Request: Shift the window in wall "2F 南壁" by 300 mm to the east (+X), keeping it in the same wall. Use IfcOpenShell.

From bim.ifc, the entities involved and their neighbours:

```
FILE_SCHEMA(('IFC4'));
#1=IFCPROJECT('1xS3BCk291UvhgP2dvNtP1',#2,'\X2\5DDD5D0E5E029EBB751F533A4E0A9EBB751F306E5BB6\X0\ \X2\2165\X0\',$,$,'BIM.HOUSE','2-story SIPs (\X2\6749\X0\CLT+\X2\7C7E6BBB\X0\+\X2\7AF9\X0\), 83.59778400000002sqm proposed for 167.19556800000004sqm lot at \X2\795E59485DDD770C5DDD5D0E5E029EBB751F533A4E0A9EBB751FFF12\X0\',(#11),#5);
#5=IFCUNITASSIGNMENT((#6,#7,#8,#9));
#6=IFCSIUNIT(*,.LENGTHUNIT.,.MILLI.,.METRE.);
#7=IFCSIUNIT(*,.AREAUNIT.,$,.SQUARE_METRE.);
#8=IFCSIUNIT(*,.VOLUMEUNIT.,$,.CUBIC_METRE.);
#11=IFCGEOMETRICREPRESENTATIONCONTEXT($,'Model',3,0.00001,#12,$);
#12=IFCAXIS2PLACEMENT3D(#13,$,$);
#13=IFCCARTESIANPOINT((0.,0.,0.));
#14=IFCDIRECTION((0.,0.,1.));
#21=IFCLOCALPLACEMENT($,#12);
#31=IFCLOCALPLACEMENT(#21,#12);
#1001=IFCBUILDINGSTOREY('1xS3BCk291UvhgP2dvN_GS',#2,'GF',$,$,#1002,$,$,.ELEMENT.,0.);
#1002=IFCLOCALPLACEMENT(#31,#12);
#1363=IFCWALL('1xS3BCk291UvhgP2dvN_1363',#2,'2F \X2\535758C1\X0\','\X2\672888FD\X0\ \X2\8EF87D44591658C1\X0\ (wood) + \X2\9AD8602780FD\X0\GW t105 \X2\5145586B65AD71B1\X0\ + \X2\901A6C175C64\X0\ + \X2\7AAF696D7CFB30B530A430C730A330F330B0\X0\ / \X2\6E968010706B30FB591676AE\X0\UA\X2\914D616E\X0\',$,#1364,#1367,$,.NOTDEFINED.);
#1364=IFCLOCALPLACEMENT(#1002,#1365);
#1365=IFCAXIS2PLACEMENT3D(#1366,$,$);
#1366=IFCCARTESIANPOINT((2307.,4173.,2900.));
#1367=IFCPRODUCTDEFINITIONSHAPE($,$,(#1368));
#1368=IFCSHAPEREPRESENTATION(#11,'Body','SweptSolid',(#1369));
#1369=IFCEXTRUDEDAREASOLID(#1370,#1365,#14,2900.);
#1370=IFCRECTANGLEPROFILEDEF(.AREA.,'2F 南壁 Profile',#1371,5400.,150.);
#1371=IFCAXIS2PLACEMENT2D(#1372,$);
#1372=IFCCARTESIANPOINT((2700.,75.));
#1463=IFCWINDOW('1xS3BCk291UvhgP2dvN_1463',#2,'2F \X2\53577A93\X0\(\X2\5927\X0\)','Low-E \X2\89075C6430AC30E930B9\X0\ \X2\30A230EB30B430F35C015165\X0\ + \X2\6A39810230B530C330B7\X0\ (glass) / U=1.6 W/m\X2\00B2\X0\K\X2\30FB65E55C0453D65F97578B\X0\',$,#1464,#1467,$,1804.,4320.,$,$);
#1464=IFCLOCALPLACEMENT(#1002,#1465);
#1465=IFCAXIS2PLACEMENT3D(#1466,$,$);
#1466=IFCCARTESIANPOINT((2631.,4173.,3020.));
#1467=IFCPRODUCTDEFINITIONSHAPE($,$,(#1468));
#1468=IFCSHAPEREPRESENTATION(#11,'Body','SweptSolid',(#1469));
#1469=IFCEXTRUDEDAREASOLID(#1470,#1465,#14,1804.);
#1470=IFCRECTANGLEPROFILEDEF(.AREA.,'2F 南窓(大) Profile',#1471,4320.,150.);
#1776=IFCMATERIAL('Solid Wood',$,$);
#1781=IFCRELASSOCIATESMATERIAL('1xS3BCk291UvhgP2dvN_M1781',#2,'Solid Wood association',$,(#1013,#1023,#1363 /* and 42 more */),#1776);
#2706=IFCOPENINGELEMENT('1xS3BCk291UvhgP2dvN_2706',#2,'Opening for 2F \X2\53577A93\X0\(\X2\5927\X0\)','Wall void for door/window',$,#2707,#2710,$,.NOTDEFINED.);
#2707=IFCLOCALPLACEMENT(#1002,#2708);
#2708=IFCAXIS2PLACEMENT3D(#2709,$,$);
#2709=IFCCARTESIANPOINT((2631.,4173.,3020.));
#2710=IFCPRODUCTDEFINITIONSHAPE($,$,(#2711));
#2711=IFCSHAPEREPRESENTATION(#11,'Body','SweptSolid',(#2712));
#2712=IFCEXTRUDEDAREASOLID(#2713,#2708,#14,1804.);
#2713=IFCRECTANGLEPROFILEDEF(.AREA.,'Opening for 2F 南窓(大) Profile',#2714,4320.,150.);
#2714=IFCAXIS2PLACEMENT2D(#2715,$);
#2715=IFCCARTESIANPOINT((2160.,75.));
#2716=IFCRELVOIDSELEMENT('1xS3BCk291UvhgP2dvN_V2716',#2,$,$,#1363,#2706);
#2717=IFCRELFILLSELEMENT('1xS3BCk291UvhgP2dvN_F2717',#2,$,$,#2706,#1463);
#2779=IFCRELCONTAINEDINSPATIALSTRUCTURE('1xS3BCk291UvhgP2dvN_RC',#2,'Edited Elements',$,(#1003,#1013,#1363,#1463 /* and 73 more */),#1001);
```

```python
import ifcopenshell
import ifcopenshell.api.geometry
import ifcopenshell.util.placement

model = ifcopenshell.open("bim.ifc")

window = model.by_id(1463)
opening = window.FillsVoids[0].RelatingOpeningElement
wall = opening.VoidsElements[0].RelatingBuildingElement

wall_matrix = ifcopenshell.util.placement.get_local_placement(wall.ObjectPlacement)
shift = wall_matrix[:3, 0] * 300.0
before = ifcopenshell.util.placement.get_local_placement(window.ObjectPlacement)[:3, 3].copy()

# The window is not placed relative to its opening, so move both.
for product in (opening, window):
    matrix = ifcopenshell.util.placement.get_local_placement(product.ObjectPlacement)
    matrix[:3, 3] += shift
    ifcopenshell.api.geometry.edit_object_placement(model, product=product, matrix=matrix, is_si=False)

after = ifcopenshell.util.placement.get_local_placement(window.ObjectPlacement)[:3, 3]
print("window moved by", (after - before).round(3) + 0.0)

model.write("bim_updated.ifc")
```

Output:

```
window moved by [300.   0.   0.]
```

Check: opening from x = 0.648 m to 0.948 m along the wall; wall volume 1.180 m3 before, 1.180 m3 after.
